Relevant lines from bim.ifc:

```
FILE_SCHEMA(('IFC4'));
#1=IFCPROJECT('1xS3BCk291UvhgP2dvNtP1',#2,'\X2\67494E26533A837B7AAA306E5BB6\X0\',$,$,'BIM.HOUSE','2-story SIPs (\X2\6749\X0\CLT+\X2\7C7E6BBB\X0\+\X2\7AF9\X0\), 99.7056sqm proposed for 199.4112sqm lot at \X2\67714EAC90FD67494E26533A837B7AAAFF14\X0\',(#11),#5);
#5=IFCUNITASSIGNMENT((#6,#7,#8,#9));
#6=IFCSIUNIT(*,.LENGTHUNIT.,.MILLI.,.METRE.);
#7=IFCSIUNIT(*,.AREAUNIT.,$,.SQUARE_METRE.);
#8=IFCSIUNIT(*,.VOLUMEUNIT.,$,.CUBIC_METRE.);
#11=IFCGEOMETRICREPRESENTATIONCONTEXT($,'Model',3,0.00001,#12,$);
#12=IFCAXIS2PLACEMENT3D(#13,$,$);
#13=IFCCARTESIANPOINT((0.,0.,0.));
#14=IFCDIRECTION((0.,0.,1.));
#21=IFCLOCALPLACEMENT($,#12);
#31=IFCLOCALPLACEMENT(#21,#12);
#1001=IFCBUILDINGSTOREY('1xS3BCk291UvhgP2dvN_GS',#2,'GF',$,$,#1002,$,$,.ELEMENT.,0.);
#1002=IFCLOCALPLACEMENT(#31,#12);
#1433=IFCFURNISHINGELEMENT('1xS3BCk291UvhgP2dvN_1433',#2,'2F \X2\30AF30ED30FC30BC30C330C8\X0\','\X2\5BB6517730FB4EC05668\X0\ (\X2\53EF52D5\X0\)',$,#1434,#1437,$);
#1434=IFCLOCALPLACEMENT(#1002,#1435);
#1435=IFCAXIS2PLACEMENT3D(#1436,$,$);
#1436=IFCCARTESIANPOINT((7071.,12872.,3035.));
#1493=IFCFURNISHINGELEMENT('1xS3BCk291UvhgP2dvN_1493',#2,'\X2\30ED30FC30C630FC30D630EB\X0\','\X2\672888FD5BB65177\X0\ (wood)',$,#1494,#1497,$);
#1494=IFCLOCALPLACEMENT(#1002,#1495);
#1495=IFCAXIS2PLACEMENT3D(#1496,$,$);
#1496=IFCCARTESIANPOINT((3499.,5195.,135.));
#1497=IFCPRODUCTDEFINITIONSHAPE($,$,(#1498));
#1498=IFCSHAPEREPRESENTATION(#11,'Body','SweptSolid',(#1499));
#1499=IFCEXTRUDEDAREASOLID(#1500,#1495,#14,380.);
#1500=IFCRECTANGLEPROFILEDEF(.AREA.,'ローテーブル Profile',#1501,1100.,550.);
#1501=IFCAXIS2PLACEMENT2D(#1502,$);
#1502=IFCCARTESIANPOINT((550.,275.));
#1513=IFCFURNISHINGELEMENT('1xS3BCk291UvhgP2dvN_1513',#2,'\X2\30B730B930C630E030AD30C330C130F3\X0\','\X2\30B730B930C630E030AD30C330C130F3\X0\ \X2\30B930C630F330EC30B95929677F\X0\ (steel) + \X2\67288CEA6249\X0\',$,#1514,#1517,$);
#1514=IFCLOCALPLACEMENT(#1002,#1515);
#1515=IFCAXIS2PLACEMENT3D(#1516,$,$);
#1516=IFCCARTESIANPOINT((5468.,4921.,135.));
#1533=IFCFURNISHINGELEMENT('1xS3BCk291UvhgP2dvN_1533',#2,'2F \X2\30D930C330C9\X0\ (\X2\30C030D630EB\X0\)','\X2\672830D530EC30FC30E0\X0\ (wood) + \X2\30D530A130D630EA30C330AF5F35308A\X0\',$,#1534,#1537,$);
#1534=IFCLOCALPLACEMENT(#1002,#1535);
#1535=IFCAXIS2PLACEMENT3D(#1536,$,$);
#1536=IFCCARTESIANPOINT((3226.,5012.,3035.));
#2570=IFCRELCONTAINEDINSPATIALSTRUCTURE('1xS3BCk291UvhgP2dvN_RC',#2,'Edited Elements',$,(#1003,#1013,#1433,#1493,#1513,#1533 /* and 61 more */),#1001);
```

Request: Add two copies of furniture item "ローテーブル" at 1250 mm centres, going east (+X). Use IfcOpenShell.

```python
import numpy as np
import ifcopenshell
import ifcopenshell.api.geometry
import ifcopenshell.api.root
import ifcopenshell.util.element
import ifcopenshell.util.placement

model = ifcopenshell.open("bim.ifc")


def reuse_history(source, copy):
    """copy_class also copies each property set's owner history, people and application; keep the originals."""
    for rel in copy.IsDefinedBy:
        if rel.is_a("IfcRelDefinesByProperties") and (history := rel.RelatingPropertyDefinition.OwnerHistory):
            rel.RelatingPropertyDefinition.OwnerHistory = source.OwnerHistory
            ifcopenshell.util.element.remove_deep2(model, history)


source = model.by_id(1493)
base = ifcopenshell.util.placement.get_local_placement(source.ObjectPlacement)
step = np.array([1.0, 0.0, 0.0]) * 1250.0

for i in range(1, 3):
    copy = ifcopenshell.api.root.copy_class(model, product=source)
    copy.Representation = ifcopenshell.util.element.copy_deep(
        model, source.Representation, exclude=["IfcGeometricRepresentationContext", "IfcRepresentationMap"]
    )
    reuse_history(source, copy)
    matrix = base.copy()
    matrix[:3, 3] += i * step
    print("added at", matrix[:3, 3].round(3) + 0.0)
    ifcopenshell.api.geometry.edit_object_placement(model, product=copy, matrix=matrix, is_si=False)

model.write("bim_updated.ifc")
```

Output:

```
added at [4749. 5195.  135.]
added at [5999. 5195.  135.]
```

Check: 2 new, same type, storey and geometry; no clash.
